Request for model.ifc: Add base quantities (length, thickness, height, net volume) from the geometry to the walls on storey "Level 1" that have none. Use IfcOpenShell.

First a look at what the model holds.

```python
import ifcopenshell
import ifcopenshell.util.element
import ifcopenshell.util.unit

model = ifcopenshell.open("model.ifc")
print(model.schema)
for unit_type in ("LENGTHUNIT", "AREAUNIT", "VOLUMEUNIT"):
    print(unit_type, ifcopenshell.util.unit.calculate_unit_scale(model, unit_type))
storey = next(s for s in model.by_type("IfcBuildingStorey") if s.Name == "Level 1")
walls = [e for e in ifcopenshell.util.element.get_decomposition(storey) if e.is_a("IfcWall")]
for e in sorted(walls, key=lambda e: e.id()):
    print(e.id(), e.is_a(), e.Name, list(ifcopenshell.util.element.get_psets(e, qtos_only=True)), sep=" | ")
```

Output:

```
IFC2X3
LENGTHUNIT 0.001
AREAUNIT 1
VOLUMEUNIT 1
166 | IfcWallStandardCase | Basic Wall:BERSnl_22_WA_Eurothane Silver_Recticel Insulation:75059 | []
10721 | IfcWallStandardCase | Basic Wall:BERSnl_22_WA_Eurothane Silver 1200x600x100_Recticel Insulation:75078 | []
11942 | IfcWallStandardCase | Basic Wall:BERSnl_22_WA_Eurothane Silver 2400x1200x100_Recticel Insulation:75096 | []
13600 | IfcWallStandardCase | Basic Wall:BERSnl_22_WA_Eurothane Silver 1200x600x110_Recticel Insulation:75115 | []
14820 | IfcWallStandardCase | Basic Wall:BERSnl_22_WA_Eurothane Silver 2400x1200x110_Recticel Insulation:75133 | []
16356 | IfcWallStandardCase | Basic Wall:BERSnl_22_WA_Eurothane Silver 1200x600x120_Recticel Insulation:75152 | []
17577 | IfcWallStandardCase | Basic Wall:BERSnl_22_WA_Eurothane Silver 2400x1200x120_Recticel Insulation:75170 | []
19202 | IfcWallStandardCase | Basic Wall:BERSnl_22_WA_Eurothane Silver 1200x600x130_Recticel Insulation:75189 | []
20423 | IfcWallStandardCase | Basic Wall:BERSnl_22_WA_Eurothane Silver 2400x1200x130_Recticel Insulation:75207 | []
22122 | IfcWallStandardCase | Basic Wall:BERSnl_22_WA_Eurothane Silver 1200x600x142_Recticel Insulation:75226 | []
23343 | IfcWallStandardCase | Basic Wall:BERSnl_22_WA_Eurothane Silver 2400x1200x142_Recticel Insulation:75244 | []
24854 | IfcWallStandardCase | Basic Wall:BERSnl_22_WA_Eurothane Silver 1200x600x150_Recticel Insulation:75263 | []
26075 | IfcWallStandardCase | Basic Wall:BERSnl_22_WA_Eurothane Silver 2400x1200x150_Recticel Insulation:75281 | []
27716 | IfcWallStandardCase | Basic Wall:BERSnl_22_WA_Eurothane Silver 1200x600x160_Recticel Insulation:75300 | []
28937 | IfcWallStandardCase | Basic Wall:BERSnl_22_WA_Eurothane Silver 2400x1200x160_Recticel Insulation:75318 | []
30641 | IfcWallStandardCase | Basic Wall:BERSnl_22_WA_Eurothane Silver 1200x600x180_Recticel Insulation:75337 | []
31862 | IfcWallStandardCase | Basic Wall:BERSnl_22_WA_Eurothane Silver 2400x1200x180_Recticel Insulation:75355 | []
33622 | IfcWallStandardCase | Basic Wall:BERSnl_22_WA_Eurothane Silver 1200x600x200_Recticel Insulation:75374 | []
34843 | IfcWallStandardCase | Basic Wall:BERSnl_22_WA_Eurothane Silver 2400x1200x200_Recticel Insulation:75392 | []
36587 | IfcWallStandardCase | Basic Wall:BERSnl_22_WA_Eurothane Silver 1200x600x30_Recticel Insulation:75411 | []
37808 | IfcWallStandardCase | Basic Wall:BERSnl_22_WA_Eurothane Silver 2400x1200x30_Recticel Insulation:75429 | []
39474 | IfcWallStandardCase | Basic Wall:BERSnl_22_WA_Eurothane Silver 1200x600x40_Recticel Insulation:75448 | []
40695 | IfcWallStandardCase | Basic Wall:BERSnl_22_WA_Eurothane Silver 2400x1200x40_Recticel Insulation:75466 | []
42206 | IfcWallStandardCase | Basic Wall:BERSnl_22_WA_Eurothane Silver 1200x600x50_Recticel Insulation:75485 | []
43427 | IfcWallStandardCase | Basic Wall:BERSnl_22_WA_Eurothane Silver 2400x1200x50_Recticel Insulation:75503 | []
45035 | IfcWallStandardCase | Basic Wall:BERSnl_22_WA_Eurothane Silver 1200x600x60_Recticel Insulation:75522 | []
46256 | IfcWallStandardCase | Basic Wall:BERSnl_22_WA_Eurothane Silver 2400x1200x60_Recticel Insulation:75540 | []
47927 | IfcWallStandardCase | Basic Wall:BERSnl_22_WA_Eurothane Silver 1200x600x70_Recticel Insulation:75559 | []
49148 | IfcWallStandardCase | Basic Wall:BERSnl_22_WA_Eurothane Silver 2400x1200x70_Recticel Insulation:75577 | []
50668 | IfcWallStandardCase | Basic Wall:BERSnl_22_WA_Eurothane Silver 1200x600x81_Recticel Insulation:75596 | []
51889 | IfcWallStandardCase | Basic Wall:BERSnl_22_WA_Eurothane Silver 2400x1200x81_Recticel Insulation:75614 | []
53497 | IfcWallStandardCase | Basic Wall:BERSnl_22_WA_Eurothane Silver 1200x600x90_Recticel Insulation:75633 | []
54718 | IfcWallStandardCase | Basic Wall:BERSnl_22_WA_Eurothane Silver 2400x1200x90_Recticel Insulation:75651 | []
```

```python
import ifcopenshell
import ifcopenshell.api.pset
import ifcopenshell.geom
import ifcopenshell.util.element
import ifcopenshell.util.shape
import ifcopenshell.util.unit

model = ifcopenshell.open("model.ifc")
unit_scale = ifcopenshell.util.unit.calculate_unit_scale(model)
volume_scale = ifcopenshell.util.unit.calculate_unit_scale(model, "VOLUMEUNIT")
settings = ifcopenshell.geom.settings()

storey = next(s for s in model.by_type("IfcBuildingStorey") if s.Name == "Level 1")
walls = [e for e in ifcopenshell.util.element.get_decomposition(storey) if e.is_a("IfcWall")]

for e in sorted(walls, key=lambda e: e.id()):
    if ifcopenshell.util.element.get_psets(e, qtos_only=True, should_inherit=False):
        continue
    # Geometry comes back in metres, in the element's own axes.
    shape = ifcopenshell.geom.create_shape(settings, e)
    values = {
        "Length": ifcopenshell.util.shape.get_x(shape.geometry) / unit_scale,
        "Width": ifcopenshell.util.shape.get_y(shape.geometry) / unit_scale,
        "Height": ifcopenshell.util.shape.get_z(shape.geometry) / unit_scale,
        "NetVolume": ifcopenshell.util.shape.get_volume(shape.geometry) / volume_scale,
    }
    qto = ifcopenshell.api.pset.add_qto(model, product=e, name="BaseQuantities")
    ifcopenshell.api.pset.edit_qto(model, qto=qto, properties=values)
    print(e.id(), {k: round(v, 3) for k, v in values.items()})

model.write("model_v2.ifc")
```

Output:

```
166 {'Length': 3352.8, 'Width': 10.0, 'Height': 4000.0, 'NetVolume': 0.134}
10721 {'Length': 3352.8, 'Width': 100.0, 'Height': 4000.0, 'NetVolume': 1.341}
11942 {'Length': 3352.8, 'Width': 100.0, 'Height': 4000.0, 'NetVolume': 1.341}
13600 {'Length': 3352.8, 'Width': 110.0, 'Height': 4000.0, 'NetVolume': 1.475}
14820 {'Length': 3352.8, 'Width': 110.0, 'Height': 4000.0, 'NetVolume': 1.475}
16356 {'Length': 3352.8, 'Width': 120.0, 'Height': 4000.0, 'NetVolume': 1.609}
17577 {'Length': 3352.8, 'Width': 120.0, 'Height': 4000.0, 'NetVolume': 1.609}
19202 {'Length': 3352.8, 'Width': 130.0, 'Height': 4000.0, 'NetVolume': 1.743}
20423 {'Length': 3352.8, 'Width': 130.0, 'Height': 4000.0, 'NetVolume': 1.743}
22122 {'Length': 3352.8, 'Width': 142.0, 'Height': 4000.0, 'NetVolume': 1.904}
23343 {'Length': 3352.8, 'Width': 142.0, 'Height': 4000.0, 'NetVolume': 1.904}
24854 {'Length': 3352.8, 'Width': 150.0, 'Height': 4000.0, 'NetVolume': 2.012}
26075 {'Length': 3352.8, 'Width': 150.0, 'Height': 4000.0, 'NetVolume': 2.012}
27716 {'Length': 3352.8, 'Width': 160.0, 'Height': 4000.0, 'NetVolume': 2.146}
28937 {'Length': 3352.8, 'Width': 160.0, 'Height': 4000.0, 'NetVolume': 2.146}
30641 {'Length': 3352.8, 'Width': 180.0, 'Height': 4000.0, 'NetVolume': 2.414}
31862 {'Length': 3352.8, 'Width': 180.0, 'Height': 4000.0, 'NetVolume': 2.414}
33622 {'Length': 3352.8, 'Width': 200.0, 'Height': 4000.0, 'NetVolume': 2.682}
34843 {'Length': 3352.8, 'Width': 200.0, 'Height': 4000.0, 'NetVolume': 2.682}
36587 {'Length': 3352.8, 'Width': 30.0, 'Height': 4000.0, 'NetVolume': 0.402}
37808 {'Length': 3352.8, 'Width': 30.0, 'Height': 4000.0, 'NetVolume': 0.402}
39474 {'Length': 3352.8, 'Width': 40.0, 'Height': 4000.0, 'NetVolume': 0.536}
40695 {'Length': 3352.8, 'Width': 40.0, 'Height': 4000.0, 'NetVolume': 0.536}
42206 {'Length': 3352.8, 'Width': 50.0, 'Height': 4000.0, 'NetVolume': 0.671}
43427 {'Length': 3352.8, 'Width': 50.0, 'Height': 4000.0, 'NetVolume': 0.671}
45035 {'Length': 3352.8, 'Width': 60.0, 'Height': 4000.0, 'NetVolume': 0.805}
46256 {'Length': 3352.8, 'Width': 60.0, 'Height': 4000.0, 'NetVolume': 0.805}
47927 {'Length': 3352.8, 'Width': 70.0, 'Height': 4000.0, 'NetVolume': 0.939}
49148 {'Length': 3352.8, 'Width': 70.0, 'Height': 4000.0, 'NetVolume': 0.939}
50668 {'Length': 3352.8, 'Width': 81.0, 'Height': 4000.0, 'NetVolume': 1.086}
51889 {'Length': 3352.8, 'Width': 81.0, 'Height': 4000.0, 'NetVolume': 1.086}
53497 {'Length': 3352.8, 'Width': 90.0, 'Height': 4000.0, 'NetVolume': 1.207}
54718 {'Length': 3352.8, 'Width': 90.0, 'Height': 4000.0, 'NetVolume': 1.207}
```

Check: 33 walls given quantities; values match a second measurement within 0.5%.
